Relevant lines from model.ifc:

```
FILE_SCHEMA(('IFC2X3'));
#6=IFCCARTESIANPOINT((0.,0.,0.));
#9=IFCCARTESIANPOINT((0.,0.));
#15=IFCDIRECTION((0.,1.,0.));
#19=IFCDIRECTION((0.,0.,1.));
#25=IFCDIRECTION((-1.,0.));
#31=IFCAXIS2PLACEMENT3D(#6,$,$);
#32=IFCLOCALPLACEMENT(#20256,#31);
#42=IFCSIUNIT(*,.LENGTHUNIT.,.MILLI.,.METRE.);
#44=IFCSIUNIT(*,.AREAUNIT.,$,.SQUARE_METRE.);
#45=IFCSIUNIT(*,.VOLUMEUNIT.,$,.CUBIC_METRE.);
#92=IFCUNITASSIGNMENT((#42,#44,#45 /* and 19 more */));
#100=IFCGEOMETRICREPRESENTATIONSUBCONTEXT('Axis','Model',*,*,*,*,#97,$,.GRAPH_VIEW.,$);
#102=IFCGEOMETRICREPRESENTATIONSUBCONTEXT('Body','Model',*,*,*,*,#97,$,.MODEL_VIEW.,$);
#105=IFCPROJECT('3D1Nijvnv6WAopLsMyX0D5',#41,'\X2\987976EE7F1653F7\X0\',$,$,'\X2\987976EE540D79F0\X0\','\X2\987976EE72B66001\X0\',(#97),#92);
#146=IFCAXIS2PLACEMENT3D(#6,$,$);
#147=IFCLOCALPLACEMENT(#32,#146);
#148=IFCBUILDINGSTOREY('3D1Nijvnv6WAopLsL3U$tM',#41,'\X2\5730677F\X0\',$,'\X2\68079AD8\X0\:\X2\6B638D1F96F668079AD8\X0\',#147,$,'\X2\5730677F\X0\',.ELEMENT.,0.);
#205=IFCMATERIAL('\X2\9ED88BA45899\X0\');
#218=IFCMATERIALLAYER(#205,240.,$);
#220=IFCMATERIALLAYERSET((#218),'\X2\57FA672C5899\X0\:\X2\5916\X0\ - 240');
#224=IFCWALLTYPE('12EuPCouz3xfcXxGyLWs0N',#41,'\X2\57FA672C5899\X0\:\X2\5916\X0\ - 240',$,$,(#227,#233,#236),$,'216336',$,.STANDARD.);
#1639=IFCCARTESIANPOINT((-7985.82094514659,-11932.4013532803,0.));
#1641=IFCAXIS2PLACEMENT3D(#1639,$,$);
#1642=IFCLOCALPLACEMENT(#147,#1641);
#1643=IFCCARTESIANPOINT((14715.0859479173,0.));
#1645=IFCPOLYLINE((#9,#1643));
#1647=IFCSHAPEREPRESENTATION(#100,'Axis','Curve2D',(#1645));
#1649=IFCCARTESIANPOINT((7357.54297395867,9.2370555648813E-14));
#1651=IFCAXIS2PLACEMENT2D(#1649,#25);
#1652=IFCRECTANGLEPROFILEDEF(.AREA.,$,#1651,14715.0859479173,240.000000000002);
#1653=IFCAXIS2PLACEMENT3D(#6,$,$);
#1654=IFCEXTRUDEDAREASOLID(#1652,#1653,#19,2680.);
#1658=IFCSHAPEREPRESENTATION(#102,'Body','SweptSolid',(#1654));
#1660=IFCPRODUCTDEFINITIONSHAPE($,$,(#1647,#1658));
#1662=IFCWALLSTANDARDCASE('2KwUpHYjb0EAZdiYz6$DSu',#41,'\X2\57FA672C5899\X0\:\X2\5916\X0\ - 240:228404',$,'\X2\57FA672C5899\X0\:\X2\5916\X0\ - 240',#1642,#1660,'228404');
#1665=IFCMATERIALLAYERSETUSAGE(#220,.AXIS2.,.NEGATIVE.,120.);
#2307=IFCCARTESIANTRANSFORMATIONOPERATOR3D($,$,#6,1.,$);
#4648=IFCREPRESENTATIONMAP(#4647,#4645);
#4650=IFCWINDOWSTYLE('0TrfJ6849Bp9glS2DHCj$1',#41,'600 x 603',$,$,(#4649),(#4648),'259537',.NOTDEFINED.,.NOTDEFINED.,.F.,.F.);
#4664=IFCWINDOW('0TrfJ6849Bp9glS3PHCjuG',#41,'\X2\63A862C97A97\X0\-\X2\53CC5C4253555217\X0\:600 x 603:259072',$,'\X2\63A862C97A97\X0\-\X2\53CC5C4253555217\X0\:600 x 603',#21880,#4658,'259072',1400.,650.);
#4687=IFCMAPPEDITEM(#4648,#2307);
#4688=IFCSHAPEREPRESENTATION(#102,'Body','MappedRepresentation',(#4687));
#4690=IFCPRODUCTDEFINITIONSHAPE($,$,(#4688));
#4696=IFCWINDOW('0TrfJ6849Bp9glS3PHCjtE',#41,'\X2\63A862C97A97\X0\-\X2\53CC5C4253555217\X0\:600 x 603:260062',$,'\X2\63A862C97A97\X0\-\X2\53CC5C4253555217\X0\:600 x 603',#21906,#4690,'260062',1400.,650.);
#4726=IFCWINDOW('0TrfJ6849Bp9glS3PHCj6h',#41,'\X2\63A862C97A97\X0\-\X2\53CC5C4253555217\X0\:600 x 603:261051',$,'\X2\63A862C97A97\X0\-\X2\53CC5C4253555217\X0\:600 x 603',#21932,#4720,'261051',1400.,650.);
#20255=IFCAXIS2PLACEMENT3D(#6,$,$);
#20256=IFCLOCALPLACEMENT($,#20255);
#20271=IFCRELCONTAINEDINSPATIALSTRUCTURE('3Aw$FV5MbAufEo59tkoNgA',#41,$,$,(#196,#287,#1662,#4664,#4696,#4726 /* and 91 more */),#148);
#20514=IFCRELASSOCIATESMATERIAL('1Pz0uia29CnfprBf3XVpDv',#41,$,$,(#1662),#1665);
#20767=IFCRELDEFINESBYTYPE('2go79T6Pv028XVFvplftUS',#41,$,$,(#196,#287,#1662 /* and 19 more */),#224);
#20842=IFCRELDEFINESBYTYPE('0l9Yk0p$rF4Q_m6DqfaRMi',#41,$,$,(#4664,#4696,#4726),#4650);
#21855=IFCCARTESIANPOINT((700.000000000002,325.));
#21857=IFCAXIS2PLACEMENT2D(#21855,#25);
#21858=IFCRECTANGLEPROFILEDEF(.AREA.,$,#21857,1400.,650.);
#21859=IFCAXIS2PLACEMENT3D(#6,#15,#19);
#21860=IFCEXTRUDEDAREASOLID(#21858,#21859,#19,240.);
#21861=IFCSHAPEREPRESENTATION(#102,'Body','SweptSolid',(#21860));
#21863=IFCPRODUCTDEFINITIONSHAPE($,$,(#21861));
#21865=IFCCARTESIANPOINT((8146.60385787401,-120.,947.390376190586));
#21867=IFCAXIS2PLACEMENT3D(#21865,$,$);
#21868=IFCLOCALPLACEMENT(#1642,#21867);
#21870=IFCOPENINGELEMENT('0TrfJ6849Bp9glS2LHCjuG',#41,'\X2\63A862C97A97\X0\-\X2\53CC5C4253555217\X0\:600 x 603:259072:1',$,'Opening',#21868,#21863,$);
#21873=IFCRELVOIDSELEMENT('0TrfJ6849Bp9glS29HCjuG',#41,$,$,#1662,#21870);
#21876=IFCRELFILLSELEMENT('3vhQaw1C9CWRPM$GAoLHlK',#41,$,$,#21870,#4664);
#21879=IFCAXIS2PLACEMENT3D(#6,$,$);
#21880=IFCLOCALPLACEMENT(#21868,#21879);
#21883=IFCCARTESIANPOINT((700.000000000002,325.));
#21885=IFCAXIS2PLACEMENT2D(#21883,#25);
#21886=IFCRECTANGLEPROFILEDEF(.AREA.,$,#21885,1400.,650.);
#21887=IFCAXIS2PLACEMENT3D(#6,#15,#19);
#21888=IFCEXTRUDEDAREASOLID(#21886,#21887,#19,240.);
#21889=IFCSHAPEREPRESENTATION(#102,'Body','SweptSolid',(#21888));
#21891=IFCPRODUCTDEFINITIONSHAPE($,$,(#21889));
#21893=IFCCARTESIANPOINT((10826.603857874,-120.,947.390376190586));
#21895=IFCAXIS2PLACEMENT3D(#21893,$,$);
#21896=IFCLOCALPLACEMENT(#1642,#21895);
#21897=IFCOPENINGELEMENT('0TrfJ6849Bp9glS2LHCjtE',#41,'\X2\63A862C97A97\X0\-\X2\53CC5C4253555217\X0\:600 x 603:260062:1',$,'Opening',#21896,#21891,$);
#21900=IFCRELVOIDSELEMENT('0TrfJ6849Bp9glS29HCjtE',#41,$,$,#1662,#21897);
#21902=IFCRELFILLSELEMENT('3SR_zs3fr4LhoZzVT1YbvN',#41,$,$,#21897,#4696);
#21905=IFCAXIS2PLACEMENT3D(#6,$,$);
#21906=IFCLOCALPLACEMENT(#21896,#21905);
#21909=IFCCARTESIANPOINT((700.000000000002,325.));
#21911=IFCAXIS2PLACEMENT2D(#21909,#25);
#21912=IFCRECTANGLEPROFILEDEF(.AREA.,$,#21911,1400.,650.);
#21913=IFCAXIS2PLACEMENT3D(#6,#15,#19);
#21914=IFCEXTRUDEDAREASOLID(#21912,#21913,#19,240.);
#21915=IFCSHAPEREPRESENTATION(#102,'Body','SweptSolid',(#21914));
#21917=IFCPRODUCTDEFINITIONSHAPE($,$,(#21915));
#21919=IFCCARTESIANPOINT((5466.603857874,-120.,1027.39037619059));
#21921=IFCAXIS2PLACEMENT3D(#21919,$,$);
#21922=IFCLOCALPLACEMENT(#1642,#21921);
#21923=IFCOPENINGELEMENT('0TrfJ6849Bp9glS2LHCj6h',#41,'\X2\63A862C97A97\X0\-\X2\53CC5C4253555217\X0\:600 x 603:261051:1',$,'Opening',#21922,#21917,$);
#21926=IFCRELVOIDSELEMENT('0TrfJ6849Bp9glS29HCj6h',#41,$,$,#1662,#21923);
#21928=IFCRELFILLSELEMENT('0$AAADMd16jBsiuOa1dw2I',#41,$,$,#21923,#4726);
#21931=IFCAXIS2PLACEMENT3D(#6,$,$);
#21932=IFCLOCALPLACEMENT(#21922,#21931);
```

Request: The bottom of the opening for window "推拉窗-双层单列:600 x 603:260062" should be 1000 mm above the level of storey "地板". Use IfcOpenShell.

```python
import numpy as np
import ifcopenshell
import ifcopenshell.api.geometry
import ifcopenshell.geom
import ifcopenshell.util.element
import ifcopenshell.util.placement
import ifcopenshell.util.shape
import ifcopenshell.util.unit

model = ifcopenshell.open("model.ifc")
unit_scale = ifcopenshell.util.unit.calculate_unit_scale(model)

window = model.by_guid("0TrfJ6849Bp9glS3PHCjtE")
opening = window.FillsVoids[0].RelatingOpeningElement
storey = ifcopenshell.util.element.get_container(window, ifc_class="IfcBuildingStorey")
level = ifcopenshell.util.placement.get_local_placement(storey.ObjectPlacement)[2, 3]

# The opening's origin need not be at the sill, so measure its lowest point.
shape = ifcopenshell.geom.create_shape(ifcopenshell.geom.settings(), opening)
bottom = ifcopenshell.util.shape.get_shape_bottom_elevation(shape, shape.geometry) / unit_scale
dz = level + 1 / unit_scale - bottom

shift = np.array([0.0, 0.0, dz])
# The window is placed relative to its opening, so it follows when the opening moves.
matrix = ifcopenshell.util.placement.get_local_placement(opening.ObjectPlacement)
matrix[:3, 3] += shift
ifcopenshell.api.geometry.edit_object_placement(
    model, product=opening, matrix=matrix, is_si=False, should_transform_children=True
)

print(f"moved by {dz * unit_scale:+.3f} m")

model.write("model_rev.ifc")
```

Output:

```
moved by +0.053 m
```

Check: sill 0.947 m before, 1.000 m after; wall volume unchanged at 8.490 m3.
